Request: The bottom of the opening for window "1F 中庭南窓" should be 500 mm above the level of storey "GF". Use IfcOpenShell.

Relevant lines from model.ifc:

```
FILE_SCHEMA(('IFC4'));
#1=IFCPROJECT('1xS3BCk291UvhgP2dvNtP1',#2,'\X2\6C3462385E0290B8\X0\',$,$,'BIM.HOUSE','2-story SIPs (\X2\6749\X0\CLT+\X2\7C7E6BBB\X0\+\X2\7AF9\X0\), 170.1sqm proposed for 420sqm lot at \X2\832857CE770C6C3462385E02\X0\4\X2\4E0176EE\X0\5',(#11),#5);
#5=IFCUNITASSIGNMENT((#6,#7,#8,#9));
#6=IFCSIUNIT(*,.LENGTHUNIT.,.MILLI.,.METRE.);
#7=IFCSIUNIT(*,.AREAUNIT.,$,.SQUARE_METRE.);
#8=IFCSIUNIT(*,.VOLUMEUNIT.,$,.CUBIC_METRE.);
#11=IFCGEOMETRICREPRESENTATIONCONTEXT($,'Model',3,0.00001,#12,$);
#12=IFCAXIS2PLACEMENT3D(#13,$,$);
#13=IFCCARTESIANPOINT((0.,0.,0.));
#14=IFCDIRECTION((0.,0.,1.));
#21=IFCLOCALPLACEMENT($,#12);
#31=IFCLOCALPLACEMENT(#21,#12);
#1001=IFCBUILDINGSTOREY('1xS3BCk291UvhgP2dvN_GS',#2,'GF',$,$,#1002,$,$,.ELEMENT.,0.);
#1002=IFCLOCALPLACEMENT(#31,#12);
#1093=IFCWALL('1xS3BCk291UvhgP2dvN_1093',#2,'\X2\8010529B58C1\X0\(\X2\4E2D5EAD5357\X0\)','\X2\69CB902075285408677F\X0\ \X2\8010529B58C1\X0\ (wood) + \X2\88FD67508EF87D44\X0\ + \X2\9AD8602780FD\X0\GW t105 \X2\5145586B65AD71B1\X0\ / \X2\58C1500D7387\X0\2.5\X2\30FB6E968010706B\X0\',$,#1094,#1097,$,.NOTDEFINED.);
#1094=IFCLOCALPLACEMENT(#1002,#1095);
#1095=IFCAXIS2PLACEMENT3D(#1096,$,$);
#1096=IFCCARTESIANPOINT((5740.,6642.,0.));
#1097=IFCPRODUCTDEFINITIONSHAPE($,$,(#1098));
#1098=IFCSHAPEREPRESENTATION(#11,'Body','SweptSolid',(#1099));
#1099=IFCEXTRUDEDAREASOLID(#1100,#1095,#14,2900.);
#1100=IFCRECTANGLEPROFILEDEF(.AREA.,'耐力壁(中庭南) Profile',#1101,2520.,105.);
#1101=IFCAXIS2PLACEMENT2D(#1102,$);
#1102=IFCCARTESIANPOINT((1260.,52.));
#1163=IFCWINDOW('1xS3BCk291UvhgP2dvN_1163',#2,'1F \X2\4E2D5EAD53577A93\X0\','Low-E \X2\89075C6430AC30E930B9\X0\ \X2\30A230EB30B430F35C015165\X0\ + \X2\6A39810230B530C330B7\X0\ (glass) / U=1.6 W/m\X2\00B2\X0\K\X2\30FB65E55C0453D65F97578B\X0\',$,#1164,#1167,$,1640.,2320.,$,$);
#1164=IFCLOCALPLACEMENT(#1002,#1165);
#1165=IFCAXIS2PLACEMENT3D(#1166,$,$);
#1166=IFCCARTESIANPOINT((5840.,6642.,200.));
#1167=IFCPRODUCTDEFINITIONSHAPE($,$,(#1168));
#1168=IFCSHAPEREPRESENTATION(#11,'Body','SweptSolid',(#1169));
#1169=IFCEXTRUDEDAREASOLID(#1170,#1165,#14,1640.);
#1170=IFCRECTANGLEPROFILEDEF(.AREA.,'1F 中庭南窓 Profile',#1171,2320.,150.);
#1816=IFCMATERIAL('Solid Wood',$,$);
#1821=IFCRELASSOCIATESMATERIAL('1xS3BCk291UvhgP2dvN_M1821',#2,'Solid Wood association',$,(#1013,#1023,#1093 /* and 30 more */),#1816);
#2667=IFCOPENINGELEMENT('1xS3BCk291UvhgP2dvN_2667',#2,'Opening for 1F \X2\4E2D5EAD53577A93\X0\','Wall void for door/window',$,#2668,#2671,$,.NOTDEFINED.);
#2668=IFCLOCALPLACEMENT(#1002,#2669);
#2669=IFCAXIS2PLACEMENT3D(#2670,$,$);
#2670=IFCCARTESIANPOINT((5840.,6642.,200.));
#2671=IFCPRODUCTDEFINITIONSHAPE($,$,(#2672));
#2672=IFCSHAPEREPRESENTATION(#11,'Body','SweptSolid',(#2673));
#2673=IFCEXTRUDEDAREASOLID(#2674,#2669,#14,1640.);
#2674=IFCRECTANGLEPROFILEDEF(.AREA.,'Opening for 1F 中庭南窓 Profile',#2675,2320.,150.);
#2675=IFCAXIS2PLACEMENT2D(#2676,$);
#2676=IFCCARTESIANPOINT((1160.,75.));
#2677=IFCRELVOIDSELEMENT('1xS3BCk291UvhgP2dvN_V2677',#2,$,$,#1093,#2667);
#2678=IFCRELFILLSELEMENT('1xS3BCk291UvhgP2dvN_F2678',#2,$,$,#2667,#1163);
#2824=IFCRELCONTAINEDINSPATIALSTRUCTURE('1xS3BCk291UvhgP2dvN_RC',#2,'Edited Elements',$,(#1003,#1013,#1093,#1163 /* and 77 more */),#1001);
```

```python
import numpy as np
import ifcopenshell
import ifcopenshell.api.geometry
import ifcopenshell.geom
import ifcopenshell.util.element
import ifcopenshell.util.placement
import ifcopenshell.util.shape
import ifcopenshell.util.unit

model = ifcopenshell.open("model.ifc")
unit_scale = ifcopenshell.util.unit.calculate_unit_scale(model)

window = model.by_id(1163)
opening = window.FillsVoids[0].RelatingOpeningElement
storey = ifcopenshell.util.element.get_container(window, ifc_class="IfcBuildingStorey")
level = ifcopenshell.util.placement.get_local_placement(storey.ObjectPlacement)[2, 3]

# The opening's origin need not be at the sill, so measure its lowest point.
shape = ifcopenshell.geom.create_shape(ifcopenshell.geom.settings(), opening)
bottom = ifcopenshell.util.shape.get_shape_bottom_elevation(shape, shape.geometry) / unit_scale
dz = level + 500.0 - bottom

shift = np.array([0.0, 0.0, dz])
# The window is not placed relative to its opening, so move both.
for product in (opening, window):
    matrix = ifcopenshell.util.placement.get_local_placement(product.ObjectPlacement)
    matrix[:3, 3] += shift
    ifcopenshell.api.geometry.edit_object_placement(model, product=product, matrix=matrix, is_si=False)

print(f"moved by {dz * unit_scale:+.3f} m")

model.write("model_edited.ifc")
```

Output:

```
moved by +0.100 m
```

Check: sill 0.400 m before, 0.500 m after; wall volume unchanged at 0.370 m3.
